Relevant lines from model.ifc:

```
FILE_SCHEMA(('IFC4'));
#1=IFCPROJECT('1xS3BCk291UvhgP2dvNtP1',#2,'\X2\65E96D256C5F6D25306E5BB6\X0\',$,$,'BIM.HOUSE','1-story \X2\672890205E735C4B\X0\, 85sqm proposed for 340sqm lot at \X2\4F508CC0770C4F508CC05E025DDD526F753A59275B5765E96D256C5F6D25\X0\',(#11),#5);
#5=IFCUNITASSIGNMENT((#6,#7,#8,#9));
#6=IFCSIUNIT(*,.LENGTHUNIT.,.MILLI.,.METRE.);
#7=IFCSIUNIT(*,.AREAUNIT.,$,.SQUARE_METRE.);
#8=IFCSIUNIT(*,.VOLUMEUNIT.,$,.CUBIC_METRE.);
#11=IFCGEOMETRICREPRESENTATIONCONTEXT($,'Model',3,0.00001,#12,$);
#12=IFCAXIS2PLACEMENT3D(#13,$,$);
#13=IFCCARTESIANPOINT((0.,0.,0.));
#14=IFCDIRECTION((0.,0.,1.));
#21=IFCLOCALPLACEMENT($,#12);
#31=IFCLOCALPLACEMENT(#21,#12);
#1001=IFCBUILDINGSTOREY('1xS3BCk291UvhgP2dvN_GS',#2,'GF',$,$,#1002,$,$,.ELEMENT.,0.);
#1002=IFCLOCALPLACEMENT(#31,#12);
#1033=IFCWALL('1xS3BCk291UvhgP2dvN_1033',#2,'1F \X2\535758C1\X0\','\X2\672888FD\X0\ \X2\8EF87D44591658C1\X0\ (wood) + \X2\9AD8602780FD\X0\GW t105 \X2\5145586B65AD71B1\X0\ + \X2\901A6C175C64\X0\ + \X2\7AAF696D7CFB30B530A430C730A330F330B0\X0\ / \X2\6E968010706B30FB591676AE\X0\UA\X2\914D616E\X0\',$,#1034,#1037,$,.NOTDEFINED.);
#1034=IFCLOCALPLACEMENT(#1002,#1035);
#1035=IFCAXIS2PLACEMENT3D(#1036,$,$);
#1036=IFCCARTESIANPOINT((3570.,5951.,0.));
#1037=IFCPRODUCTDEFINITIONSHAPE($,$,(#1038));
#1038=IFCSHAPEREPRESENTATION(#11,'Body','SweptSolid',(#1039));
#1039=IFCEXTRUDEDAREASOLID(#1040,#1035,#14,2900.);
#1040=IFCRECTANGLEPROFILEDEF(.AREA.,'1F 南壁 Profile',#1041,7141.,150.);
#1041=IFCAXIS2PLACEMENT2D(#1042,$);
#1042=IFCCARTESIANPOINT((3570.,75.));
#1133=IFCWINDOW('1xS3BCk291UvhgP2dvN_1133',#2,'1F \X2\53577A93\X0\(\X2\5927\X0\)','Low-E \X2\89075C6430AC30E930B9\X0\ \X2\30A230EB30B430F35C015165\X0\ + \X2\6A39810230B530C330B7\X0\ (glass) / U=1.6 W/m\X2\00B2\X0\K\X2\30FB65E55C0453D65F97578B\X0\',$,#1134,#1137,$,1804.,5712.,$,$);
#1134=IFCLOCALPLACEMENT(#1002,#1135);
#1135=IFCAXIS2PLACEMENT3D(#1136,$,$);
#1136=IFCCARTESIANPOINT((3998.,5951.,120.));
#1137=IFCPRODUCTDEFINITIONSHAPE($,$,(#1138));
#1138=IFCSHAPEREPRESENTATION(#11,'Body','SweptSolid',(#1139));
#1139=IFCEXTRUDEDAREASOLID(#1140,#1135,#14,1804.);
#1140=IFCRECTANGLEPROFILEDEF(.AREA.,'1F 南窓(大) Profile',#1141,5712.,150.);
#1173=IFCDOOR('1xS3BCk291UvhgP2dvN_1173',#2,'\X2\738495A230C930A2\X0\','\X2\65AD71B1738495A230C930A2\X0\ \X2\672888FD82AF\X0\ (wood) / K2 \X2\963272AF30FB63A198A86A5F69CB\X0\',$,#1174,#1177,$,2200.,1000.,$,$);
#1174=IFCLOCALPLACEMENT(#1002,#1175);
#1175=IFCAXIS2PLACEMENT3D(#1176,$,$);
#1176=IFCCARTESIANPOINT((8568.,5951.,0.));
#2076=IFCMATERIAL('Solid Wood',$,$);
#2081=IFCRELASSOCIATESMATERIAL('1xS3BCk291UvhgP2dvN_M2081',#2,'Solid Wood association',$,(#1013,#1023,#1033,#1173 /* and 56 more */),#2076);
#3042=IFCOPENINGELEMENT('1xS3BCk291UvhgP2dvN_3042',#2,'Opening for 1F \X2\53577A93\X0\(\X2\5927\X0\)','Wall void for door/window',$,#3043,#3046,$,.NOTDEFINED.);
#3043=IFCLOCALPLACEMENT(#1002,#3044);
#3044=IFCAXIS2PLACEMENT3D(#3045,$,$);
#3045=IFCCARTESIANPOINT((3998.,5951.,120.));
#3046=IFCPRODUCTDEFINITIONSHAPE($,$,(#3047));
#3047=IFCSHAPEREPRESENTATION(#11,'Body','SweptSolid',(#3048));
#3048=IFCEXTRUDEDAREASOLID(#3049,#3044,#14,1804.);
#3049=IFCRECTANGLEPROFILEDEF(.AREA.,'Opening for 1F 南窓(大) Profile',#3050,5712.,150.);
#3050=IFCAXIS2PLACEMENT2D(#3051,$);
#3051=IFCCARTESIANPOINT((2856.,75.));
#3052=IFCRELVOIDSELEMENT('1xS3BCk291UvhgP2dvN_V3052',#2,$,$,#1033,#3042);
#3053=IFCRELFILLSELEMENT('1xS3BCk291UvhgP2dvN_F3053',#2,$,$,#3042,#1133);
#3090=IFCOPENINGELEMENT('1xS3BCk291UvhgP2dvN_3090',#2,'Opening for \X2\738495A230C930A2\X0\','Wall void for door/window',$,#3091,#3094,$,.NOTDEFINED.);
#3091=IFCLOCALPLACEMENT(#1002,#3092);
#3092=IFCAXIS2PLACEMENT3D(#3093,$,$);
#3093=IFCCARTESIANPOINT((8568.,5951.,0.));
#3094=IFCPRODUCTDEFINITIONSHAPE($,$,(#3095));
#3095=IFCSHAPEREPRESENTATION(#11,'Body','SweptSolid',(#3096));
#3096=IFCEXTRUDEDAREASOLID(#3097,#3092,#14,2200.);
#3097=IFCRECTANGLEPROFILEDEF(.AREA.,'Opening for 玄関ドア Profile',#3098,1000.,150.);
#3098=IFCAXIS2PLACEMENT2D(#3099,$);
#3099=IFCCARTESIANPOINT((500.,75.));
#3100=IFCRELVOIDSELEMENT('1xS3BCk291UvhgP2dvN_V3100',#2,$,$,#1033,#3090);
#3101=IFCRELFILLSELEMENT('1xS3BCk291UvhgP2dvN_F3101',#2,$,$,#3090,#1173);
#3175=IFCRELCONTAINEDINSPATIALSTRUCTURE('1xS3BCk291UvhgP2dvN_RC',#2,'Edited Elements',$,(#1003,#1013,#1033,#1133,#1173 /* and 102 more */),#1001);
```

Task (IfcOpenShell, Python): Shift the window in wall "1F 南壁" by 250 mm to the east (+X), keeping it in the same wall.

```python
import ifcopenshell
import ifcopenshell.api.geometry
import ifcopenshell.util.placement

model = ifcopenshell.open("model.ifc")

window = model.by_guid("1xS3BCk291UvhgP2dvN_1133")
opening = window.FillsVoids[0].RelatingOpeningElement
wall = opening.VoidsElements[0].RelatingBuildingElement

wall_matrix = ifcopenshell.util.placement.get_local_placement(wall.ObjectPlacement)
shift = wall_matrix[:3, 0] * 250.0
before = ifcopenshell.util.placement.get_local_placement(window.ObjectPlacement)[:3, 3].copy()

# The window is not placed relative to its opening, so move both.
for product in (opening, window):
    matrix = ifcopenshell.util.placement.get_local_placement(product.ObjectPlacement)
    matrix[:3, 3] += shift
    ifcopenshell.api.geometry.edit_object_placement(model, product=product, matrix=matrix, is_si=False)

after = ifcopenshell.util.placement.get_local_placement(window.ObjectPlacement)[:3, 3]
print("window moved by", (after - before).round(3) + 0.0)

model.write("model_updated.ifc")
```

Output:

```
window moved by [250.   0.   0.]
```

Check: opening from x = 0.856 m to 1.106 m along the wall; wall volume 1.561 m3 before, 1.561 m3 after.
